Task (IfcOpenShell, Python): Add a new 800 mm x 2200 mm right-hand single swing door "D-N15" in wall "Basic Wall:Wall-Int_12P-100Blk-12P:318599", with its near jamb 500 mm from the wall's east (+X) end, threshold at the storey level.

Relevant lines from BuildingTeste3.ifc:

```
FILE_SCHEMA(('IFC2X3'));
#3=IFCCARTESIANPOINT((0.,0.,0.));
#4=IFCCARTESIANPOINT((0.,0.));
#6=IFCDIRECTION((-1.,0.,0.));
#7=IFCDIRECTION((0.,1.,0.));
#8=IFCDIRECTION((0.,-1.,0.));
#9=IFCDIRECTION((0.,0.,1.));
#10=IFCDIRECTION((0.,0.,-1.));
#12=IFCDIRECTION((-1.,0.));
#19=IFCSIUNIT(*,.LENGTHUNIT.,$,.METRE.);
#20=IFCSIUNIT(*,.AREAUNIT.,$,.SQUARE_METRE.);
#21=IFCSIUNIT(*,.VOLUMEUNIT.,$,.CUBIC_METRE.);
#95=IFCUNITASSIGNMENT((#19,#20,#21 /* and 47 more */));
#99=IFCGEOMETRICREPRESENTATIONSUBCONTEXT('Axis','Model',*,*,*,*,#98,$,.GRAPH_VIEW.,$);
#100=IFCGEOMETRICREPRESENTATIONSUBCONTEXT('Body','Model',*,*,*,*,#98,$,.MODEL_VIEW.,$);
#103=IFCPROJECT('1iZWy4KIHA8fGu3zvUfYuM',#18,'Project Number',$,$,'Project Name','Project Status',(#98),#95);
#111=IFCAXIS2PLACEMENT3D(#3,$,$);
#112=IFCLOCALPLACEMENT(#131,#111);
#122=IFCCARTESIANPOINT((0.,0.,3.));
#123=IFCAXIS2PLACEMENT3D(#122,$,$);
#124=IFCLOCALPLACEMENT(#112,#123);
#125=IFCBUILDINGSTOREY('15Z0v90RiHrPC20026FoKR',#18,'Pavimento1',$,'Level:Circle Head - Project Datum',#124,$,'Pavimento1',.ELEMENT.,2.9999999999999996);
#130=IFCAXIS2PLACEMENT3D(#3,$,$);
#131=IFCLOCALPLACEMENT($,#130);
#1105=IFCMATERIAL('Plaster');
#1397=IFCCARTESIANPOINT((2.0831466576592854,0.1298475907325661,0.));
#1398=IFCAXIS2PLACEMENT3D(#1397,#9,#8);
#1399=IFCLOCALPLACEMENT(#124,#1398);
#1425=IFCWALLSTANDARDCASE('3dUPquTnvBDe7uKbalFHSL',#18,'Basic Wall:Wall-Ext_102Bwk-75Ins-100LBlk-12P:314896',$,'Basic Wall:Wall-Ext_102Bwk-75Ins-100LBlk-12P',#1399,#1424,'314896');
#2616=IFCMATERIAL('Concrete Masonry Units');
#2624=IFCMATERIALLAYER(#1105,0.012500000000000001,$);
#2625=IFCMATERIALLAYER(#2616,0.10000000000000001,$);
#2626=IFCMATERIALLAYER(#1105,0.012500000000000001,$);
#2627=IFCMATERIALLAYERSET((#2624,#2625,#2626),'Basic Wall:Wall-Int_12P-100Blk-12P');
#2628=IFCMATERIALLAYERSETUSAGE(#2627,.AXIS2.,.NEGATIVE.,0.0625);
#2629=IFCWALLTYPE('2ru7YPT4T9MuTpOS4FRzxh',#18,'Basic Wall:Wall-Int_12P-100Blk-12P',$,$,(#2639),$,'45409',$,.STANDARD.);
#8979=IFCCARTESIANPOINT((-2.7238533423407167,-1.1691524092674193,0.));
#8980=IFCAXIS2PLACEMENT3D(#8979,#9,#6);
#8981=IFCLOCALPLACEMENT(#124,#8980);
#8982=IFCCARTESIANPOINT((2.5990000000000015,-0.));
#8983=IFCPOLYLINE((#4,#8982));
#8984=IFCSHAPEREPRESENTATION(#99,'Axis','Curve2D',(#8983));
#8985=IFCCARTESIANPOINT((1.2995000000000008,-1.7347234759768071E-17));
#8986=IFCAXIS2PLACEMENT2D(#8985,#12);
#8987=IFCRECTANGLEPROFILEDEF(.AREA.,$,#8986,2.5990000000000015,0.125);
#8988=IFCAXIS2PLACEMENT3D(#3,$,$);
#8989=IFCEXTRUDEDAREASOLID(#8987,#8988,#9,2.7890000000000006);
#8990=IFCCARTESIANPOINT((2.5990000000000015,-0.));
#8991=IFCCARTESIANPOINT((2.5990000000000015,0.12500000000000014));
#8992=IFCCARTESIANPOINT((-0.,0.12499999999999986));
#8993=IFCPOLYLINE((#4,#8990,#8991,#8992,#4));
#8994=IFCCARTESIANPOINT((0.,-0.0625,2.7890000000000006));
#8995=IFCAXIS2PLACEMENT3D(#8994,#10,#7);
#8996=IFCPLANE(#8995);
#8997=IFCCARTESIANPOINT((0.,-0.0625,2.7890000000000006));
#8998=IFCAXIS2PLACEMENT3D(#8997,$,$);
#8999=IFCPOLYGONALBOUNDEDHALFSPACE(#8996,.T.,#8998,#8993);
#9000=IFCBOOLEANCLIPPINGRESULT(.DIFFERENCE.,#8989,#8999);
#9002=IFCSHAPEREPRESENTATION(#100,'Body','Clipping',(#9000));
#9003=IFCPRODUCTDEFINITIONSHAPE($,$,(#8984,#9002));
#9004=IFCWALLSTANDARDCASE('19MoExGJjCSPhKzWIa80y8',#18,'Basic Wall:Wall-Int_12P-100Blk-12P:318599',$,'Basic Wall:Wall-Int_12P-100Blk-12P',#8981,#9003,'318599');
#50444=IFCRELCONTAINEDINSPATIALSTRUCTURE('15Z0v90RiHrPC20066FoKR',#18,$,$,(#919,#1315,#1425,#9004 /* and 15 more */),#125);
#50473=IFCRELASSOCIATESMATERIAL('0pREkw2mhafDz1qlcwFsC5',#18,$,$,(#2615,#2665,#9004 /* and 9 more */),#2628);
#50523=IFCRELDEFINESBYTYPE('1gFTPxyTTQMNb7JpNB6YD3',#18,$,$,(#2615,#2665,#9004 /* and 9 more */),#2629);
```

```python
import numpy as np
import ifcopenshell
import ifcopenshell.api.feature
import ifcopenshell.api.geometry
import ifcopenshell.api.root
import ifcopenshell.api.spatial
import ifcopenshell.api.type
import ifcopenshell.geom
import ifcopenshell.util.element
import ifcopenshell.util.placement
import ifcopenshell.util.representation
import ifcopenshell.util.shape
import ifcopenshell.util.unit

model = ifcopenshell.open("BuildingTeste3.ifc")
unit_scale = ifcopenshell.util.unit.calculate_unit_scale(model)
settings = ifcopenshell.geom.settings()


def volume(element):
    """Net volume in cubic metres, openings subtracted."""
    shape = ifcopenshell.geom.create_shape(settings, element)
    return ifcopenshell.util.shape.get_volume(shape.geometry)


wall = model.by_guid("19MoExGJjCSPhKzWIa80y8")
storey = ifcopenshell.util.element.get_container(wall, ifc_class="IfcBuildingStorey")
context = ifcopenshell.util.representation.get_context(model, "Model", "Body", "MODEL_VIEW")
before = volume(wall)

width, height, from_end, sill = 0.8, 2.2, 0.5, 0.0  # metres

# The wall runs along its own X axis, and the end named is its -X end.
wall_shape = ifcopenshell.geom.create_shape(settings, wall)
x, y, z = ifcopenshell.util.shape.get_vertices(wall_shape.geometry).T
start = x.min() + from_end
face, thickness = float(y.min()), float(y.max() - y.min())
wall_matrix = ifcopenshell.util.placement.get_local_placement(wall.ObjectPlacement)
level = ifcopenshell.util.placement.get_local_placement(storey.ObjectPlacement)[2, 3]


def in_wall(x, y):
    """Placement at x, y metres in the wall's axes, at sill height."""
    matrix = wall_matrix.copy()
    matrix[:, 3] = wall_matrix @ np.array([x / unit_scale, y / unit_scale, 0.0, 1.0])
    matrix[2, 3] = level + sill / unit_scale
    return matrix


# Opening: a box that overshoots both wall faces by 50 mm.
opening = ifcopenshell.api.root.create_entity(model, ifc_class="IfcOpeningElement")
box = ifcopenshell.api.geometry.add_wall_representation(
    model, context=context, length=width, height=height, thickness=thickness + 0.1
)
ifcopenshell.api.geometry.assign_representation(model, product=opening, representation=box)
ifcopenshell.api.geometry.edit_object_placement(model, product=opening, matrix=in_wall(start, face - 0.05), is_si=False)
ifcopenshell.api.feature.add_feature(model, feature=opening, element=wall)

door = ifcopenshell.api.root.create_entity(model, ifc_class="IfcDoor", name="D-N15")
door.OverallWidth, door.OverallHeight = width / unit_scale, height / unit_scale
body = ifcopenshell.api.geometry.add_door_representation(
    model,
    context=context,
    overall_width=door.OverallWidth,
    overall_height=door.OverallHeight,
    operation_type="SINGLE_SWING_RIGHT",
    lining_properties={"LiningDepth": thickness / unit_scale, "ThresholdDepth": thickness / unit_scale},
)
ifcopenshell.api.geometry.assign_representation(model, product=door, representation=body)
ifcopenshell.api.spatial.assign_container(model, products=[door], relating_structure=storey)
fills = ifcopenshell.api.feature.add_filling(model, opening=opening, element=door)
fills.OwnerHistory = door.OwnerHistory  # required in IFC2X3

# IFC2X3 keeps the operation on the door style.
style = ifcopenshell.api.root.create_entity(model, ifc_class="IfcDoorStyle", name="D-N15")
style.OperationType, style.ConstructionType = "SINGLE_SWING_RIGHT", "NOTDEFINED"
style.ParameterTakesPrecedence = style.Sizeable = False
ifcopenshell.api.type.assign_type(model, related_objects=[door], relating_type=style)

# The lining spans the wall, so the door starts at the wall face.
ifcopenshell.api.geometry.edit_object_placement(model, product=door, matrix=in_wall(start, face), is_si=False)

after = volume(wall)

print(f"wall volume {before:.3f} -> {after:.3f} m3")

model.write("BuildingTeste3_updated.ifc")
```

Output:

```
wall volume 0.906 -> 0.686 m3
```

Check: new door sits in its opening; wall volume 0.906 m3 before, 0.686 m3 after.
